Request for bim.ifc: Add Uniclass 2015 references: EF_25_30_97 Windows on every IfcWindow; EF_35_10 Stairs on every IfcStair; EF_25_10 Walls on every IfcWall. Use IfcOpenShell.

First a look at what the model holds.

```python
import ifcopenshell

model = ifcopenshell.open("bim.ifc")
print(model.schema)
print("classifications:", [c.Name for c in model.by_type("IfcClassification")])
for ifc_class in ("IfcDoor", "IfcRoof", "IfcStair", "IfcWall", "IfcWindow"):
    print(ifc_class, len(model.by_type(ifc_class)))
```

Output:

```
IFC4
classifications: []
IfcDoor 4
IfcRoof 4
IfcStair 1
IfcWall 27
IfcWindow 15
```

```python
import ifcopenshell
import ifcopenshell.api.classification

model = ifcopenshell.open("bim.ifc")

system = ifcopenshell.api.classification.add_classification(model, classification="Uniclass 2015")

codes = {
    "IfcWindow": ("EF_25_30_97", "Windows"),
    "IfcStair": ("EF_35_10", "Stairs"),
    "IfcWall": ("EF_25_10", "Walls"),
}
for ifc_class, (code, name) in codes.items():
    products = model.by_type(ifc_class)
    ifcopenshell.api.classification.add_reference(
        model, products=products, classification=system, identification=code, name=name
    )
    print(code, len(products))

model.write("bim_v2.ifc")
```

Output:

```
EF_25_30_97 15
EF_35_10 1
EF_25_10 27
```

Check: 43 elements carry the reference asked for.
